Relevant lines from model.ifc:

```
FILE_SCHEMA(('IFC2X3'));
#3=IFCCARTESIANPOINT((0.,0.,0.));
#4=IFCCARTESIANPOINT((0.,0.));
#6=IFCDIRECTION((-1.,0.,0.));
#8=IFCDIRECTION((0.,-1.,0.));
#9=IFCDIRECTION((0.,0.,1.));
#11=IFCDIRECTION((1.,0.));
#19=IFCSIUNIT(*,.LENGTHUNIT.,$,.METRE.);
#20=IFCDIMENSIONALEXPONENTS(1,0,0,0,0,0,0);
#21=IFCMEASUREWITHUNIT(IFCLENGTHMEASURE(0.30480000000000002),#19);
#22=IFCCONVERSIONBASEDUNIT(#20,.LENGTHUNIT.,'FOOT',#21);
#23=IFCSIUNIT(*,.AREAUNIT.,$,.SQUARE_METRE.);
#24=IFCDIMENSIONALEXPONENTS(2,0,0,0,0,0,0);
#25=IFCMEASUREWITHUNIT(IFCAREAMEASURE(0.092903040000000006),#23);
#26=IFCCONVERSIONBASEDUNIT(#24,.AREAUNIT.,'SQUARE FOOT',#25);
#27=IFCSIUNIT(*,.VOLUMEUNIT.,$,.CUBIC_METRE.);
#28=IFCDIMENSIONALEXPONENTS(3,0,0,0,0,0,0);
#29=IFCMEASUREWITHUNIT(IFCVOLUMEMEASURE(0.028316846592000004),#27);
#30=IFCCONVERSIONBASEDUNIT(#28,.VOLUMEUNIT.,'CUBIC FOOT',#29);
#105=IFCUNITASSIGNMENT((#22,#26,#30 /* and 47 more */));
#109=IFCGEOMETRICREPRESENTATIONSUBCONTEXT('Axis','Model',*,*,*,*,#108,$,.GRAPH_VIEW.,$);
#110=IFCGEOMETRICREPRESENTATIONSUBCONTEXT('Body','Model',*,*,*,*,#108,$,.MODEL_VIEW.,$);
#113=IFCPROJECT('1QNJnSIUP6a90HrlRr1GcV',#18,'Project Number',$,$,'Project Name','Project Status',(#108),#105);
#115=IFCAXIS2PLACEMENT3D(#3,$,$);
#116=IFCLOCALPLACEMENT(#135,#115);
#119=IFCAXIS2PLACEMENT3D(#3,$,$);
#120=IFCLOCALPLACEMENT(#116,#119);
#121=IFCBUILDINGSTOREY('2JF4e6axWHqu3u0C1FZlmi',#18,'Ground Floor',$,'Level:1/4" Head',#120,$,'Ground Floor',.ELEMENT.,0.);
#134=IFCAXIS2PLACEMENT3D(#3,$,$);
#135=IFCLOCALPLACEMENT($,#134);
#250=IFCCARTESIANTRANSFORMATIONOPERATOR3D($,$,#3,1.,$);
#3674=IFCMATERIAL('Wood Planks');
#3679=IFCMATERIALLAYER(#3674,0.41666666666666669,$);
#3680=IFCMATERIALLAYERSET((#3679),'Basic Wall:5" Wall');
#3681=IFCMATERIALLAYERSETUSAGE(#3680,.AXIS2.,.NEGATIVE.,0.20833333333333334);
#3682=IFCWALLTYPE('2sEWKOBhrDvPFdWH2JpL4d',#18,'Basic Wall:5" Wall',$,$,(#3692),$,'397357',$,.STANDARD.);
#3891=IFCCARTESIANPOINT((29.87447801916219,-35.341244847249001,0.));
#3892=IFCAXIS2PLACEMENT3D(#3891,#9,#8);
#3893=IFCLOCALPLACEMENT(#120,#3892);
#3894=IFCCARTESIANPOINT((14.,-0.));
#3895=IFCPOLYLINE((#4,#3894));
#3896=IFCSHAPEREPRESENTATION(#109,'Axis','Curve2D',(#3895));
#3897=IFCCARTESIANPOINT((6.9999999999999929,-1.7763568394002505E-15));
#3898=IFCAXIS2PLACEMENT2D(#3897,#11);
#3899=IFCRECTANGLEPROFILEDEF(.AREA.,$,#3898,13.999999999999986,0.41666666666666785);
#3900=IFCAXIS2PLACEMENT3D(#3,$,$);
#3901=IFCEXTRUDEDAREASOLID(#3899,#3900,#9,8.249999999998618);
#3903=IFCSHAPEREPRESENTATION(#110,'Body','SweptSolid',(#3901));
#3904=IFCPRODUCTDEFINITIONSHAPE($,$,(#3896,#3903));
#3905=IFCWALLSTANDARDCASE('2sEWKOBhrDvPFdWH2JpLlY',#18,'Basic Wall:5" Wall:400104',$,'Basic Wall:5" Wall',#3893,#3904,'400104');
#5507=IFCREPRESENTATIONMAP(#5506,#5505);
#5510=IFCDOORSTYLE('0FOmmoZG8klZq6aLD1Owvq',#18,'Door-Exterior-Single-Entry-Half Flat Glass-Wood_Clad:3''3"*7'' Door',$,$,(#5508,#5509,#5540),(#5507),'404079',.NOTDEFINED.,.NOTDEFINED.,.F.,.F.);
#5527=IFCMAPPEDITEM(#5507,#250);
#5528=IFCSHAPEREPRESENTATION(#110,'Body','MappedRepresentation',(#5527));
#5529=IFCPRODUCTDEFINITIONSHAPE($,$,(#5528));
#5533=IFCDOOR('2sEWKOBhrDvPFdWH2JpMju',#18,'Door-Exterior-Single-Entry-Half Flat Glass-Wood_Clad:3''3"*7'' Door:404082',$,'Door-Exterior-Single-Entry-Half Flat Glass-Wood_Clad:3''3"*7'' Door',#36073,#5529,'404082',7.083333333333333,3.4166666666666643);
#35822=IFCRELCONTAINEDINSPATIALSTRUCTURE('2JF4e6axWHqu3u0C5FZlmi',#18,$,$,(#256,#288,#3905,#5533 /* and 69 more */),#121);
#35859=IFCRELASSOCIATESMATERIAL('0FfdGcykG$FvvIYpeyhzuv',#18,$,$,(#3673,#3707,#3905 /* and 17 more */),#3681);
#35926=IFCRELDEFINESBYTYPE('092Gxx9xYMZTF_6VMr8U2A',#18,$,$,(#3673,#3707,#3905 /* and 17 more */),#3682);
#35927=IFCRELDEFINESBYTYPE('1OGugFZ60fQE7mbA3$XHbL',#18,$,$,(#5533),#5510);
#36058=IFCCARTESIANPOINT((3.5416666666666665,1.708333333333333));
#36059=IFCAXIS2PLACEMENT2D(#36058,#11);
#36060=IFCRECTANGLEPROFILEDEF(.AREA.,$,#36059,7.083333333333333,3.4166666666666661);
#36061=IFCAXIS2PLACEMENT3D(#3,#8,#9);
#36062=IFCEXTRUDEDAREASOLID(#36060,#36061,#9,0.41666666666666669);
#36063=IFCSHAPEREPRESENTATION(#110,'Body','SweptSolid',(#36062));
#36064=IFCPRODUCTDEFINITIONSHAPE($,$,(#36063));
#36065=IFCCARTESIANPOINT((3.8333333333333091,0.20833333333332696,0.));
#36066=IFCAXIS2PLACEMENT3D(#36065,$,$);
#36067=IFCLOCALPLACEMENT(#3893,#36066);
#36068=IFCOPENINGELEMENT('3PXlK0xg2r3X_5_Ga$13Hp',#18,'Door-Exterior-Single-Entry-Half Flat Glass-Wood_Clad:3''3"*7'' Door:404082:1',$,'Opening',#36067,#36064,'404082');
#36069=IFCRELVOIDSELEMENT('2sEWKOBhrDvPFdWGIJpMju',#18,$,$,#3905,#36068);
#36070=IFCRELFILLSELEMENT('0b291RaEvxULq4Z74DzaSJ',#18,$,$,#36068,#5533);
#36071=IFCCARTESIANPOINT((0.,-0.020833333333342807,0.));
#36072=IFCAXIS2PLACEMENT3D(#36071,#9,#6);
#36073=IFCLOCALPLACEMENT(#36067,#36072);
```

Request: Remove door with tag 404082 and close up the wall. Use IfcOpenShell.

```python
import ifcopenshell
import ifcopenshell.api.feature
import ifcopenshell.api.root
import ifcopenshell.geom
import ifcopenshell.util.shape

model = ifcopenshell.open("model.ifc")
settings = ifcopenshell.geom.settings()


def volume(element):
    """Net volume in cubic metres, openings subtracted."""
    shape = ifcopenshell.geom.create_shape(settings, element)
    return ifcopenshell.util.shape.get_volume(shape.geometry)


door = model.by_guid("2sEWKOBhrDvPFdWH2JpMju")
opening = door.FillsVoids[0].RelatingOpeningElement
wall = opening.VoidsElements[0].RelatingBuildingElement
before = volume(wall)

ifcopenshell.api.root.remove_product(model, product=door)
ifcopenshell.api.feature.remove_feature(model, feature=opening)

after = volume(wall)

print(f"wall volume {before:.3f} -> {after:.3f} m3")

model.write("model_updated.ifc")
```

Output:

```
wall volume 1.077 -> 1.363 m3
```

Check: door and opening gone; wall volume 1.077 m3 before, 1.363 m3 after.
